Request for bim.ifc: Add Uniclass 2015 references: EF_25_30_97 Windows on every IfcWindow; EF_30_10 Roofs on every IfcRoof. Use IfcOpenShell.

First a look at what the model holds.

```python
import ifcopenshell

model = ifcopenshell.open("bim.ifc")
print(model.schema)
print("classifications:", [c.Name for c in model.by_type("IfcClassification")])
for ifc_class in ("IfcDoor", "IfcRoof", "IfcStair", "IfcWall", "IfcWindow"):
    print(ifc_class, len(model.by_type(ifc_class)))
```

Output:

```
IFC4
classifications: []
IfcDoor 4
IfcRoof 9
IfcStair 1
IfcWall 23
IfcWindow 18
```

```python
import ifcopenshell
import ifcopenshell.api.classification

model = ifcopenshell.open("bim.ifc")

system = ifcopenshell.api.classification.add_classification(model, classification="Uniclass 2015")

codes = {
    "IfcWindow": ("EF_25_30_97", "Windows"),
    "IfcRoof": ("EF_30_10", "Roofs"),
}
for ifc_class, (code, name) in codes.items():
    products = model.by_type(ifc_class)
    ifcopenshell.api.classification.add_reference(
        model, products=products, classification=system, identification=code, name=name
    )
    print(code, len(products))

model.write("bim_v2.ifc")
```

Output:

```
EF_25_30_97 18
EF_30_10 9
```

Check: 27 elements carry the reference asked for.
